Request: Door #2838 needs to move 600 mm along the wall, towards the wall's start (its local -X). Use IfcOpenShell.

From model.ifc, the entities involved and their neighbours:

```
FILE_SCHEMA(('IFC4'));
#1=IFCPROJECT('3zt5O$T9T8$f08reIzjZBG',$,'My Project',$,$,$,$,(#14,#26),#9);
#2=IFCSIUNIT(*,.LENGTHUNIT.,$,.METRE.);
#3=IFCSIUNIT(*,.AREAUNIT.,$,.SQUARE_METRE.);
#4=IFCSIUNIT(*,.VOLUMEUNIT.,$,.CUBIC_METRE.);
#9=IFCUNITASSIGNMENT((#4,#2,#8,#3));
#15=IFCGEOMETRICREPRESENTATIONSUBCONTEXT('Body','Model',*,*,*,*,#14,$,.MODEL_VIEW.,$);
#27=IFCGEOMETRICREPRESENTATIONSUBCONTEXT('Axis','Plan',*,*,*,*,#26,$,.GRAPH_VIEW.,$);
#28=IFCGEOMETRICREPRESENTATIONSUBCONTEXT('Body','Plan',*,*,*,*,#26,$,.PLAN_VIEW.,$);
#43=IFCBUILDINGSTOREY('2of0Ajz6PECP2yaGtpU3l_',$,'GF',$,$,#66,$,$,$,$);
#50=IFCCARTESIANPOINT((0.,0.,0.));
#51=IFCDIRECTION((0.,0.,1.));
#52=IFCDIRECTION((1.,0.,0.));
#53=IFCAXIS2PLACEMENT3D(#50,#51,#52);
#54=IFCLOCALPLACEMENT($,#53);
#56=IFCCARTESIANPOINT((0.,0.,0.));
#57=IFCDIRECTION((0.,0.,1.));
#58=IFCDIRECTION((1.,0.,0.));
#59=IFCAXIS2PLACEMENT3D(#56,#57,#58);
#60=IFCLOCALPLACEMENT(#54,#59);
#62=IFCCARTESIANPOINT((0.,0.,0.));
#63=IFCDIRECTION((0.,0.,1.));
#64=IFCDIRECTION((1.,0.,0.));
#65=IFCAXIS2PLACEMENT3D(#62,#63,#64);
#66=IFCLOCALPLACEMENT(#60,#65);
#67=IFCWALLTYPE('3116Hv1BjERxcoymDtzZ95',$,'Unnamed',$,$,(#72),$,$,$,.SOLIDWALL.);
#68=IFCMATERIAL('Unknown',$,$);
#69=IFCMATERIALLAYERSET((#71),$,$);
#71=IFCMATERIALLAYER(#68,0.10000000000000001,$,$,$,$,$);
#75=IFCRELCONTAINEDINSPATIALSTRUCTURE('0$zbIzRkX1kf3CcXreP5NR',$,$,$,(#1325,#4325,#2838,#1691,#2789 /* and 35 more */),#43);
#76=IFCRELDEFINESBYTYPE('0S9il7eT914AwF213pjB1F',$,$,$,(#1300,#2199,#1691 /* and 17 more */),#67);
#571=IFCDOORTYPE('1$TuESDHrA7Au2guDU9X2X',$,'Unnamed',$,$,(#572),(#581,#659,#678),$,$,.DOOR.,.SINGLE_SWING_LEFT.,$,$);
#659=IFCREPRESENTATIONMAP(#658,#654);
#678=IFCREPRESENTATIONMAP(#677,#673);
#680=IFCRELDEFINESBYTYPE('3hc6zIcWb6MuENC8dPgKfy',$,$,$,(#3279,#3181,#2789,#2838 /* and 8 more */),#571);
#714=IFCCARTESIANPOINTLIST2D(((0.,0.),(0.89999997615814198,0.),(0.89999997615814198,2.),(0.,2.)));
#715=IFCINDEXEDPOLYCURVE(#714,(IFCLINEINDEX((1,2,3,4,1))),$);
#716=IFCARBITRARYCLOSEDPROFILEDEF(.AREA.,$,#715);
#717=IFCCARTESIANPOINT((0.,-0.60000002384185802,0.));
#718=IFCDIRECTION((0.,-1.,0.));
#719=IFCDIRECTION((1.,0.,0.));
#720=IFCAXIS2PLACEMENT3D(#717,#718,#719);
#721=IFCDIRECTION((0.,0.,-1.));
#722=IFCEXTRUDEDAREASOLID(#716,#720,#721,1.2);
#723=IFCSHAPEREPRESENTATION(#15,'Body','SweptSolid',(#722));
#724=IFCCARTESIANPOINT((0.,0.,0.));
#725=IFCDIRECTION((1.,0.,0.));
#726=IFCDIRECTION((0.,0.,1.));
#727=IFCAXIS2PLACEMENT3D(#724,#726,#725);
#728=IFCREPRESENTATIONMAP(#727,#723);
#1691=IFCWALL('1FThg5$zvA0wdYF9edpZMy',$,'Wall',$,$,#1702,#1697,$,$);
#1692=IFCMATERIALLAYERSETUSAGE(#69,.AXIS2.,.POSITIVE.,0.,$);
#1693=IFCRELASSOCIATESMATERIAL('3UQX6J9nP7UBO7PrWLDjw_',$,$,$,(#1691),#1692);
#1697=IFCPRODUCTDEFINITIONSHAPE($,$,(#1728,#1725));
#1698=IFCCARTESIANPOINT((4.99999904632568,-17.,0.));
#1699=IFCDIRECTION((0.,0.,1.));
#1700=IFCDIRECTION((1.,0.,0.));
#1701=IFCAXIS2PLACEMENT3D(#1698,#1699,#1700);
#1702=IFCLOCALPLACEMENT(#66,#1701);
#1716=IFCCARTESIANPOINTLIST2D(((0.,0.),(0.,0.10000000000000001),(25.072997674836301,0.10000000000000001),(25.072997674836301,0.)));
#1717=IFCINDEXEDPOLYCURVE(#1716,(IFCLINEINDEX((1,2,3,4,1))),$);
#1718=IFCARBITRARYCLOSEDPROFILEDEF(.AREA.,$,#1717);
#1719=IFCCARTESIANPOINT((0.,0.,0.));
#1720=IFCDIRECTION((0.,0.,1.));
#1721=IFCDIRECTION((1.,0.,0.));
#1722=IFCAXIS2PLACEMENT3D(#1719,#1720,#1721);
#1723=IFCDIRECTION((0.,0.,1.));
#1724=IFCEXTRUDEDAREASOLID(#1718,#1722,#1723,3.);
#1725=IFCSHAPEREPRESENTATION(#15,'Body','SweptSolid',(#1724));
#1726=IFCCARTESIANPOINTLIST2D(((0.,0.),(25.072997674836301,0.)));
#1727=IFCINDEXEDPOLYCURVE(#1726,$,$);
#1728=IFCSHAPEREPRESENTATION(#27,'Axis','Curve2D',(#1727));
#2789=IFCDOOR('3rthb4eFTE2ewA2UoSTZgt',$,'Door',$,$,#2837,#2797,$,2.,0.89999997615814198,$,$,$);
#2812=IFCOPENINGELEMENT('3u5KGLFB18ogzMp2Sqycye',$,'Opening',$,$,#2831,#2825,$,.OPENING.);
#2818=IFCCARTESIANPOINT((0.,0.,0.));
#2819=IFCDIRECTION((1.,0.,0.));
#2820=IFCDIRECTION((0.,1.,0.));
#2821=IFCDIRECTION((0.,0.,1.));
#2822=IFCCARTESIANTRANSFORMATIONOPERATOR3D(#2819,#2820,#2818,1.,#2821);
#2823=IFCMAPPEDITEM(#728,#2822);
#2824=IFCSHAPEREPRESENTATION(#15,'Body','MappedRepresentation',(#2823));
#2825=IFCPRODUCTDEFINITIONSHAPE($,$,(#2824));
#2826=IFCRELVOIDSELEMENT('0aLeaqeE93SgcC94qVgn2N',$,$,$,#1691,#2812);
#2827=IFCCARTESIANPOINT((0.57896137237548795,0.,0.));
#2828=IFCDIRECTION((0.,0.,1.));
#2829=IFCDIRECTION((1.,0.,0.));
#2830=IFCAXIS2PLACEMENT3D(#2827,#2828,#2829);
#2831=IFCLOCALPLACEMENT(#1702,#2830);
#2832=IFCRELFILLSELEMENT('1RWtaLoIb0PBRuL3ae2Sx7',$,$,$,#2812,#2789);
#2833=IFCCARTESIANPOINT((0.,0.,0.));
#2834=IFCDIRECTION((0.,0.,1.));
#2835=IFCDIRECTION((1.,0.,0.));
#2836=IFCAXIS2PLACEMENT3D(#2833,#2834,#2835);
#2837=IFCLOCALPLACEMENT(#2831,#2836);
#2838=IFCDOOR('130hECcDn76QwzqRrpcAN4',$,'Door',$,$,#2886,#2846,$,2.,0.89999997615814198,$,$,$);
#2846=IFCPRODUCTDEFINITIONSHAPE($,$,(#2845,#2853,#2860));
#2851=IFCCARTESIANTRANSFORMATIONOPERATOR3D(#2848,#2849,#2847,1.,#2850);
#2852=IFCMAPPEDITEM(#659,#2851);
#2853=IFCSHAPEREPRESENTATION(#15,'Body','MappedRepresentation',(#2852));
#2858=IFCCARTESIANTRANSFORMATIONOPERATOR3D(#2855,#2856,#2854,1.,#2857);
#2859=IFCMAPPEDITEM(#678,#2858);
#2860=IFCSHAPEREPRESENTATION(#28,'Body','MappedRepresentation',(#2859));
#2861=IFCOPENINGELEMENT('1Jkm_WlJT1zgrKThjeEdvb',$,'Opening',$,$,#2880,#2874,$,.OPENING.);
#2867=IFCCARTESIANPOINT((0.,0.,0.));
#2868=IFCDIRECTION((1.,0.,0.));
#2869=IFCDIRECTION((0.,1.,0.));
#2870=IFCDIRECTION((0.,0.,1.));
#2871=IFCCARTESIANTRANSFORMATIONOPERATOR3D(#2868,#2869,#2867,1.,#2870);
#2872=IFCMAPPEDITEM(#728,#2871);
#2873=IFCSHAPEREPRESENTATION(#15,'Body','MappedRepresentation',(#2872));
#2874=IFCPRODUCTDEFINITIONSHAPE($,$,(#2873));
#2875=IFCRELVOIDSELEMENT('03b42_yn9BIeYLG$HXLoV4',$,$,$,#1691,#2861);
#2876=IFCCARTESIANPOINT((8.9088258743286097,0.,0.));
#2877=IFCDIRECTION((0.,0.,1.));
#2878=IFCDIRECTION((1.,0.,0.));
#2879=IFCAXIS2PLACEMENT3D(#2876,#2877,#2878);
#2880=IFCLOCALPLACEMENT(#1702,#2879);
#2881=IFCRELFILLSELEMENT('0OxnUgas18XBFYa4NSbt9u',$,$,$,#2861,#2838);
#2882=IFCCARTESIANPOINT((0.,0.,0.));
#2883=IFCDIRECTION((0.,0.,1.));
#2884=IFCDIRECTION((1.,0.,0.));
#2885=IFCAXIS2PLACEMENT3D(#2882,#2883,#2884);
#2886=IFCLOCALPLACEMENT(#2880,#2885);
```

```python
import ifcopenshell
import ifcopenshell.api.geometry
import ifcopenshell.util.placement
import ifcopenshell.util.unit

model = ifcopenshell.open("model.ifc")
unit_scale = ifcopenshell.util.unit.calculate_unit_scale(model)

door = model.by_id(2838)
opening = door.FillsVoids[0].RelatingOpeningElement
wall = opening.VoidsElements[0].RelatingBuildingElement

wall_matrix = ifcopenshell.util.placement.get_local_placement(wall.ObjectPlacement)
shift = wall_matrix[:3, 0] * -0.6 / unit_scale
before = ifcopenshell.util.placement.get_local_placement(door.ObjectPlacement)[:3, 3].copy()

# The door is placed relative to its opening, so it follows when the opening moves.
matrix = ifcopenshell.util.placement.get_local_placement(opening.ObjectPlacement)
matrix[:3, 3] += shift
ifcopenshell.api.geometry.edit_object_placement(
    model, product=opening, matrix=matrix, is_si=False, should_transform_children=True
)

after = ifcopenshell.util.placement.get_local_placement(door.ObjectPlacement)[:3, 3]
print("door moved by", (after - before).round(3) + 0.0)

model.write("model_rev.ifc")
```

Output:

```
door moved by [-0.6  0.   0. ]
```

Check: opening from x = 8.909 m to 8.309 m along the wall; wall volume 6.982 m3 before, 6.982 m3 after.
